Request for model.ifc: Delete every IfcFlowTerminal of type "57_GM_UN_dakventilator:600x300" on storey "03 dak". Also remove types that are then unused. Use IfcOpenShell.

First a look at what the model holds.

```python
import ifcopenshell
import ifcopenshell.util.element

model = ifcopenshell.open("model.ifc")
print(model.schema)
storey = next(s for s in model.by_type("IfcBuildingStorey") if s.Name == "03 dak")
terminals = [e for e in ifcopenshell.util.element.get_decomposition(storey) if e.is_a("IfcFlowTerminal")]
seen = {}
for e in terminals:
    element_type = ifcopenshell.util.element.get_type(e)
    name = element_type.Name if element_type not in (None, e) else None
    seen[name] = seen.get(name, 0) + 1
for name, count in sorted(seen.items(), key=str):
    print(count, "x", name)
```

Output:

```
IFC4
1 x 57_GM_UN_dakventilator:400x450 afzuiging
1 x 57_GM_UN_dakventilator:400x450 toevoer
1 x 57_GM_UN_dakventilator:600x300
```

```python
import ifcopenshell
import ifcopenshell.api.root
import ifcopenshell.util.element

model = ifcopenshell.open("model.ifc")

storey = next(s for s in model.by_type("IfcBuildingStorey") if s.Name == "03 dak")
terminals = [e for e in ifcopenshell.util.element.get_decomposition(storey) if e.is_a("IfcFlowTerminal")]
targets = [e for e in terminals if (t := ifcopenshell.util.element.get_type(e)) not in (None, e) and t.Name == "57_GM_UN_dakventilator:600x300"]
types = {ifcopenshell.util.element.get_type(e) for e in targets} - {None, *targets}

for e in targets:
    ifcopenshell.api.root.remove_product(model, product=e)
print(len(targets), "removed")

unused = [t for t in types if not ifcopenshell.util.element.get_types(t)]
for t in unused:
    ifcopenshell.api.root.remove_product(model, product=t)
print(len(unused), "unused types removed")

model.write("model-out.ifc")
```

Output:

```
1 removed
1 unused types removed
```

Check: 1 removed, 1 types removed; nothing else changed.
